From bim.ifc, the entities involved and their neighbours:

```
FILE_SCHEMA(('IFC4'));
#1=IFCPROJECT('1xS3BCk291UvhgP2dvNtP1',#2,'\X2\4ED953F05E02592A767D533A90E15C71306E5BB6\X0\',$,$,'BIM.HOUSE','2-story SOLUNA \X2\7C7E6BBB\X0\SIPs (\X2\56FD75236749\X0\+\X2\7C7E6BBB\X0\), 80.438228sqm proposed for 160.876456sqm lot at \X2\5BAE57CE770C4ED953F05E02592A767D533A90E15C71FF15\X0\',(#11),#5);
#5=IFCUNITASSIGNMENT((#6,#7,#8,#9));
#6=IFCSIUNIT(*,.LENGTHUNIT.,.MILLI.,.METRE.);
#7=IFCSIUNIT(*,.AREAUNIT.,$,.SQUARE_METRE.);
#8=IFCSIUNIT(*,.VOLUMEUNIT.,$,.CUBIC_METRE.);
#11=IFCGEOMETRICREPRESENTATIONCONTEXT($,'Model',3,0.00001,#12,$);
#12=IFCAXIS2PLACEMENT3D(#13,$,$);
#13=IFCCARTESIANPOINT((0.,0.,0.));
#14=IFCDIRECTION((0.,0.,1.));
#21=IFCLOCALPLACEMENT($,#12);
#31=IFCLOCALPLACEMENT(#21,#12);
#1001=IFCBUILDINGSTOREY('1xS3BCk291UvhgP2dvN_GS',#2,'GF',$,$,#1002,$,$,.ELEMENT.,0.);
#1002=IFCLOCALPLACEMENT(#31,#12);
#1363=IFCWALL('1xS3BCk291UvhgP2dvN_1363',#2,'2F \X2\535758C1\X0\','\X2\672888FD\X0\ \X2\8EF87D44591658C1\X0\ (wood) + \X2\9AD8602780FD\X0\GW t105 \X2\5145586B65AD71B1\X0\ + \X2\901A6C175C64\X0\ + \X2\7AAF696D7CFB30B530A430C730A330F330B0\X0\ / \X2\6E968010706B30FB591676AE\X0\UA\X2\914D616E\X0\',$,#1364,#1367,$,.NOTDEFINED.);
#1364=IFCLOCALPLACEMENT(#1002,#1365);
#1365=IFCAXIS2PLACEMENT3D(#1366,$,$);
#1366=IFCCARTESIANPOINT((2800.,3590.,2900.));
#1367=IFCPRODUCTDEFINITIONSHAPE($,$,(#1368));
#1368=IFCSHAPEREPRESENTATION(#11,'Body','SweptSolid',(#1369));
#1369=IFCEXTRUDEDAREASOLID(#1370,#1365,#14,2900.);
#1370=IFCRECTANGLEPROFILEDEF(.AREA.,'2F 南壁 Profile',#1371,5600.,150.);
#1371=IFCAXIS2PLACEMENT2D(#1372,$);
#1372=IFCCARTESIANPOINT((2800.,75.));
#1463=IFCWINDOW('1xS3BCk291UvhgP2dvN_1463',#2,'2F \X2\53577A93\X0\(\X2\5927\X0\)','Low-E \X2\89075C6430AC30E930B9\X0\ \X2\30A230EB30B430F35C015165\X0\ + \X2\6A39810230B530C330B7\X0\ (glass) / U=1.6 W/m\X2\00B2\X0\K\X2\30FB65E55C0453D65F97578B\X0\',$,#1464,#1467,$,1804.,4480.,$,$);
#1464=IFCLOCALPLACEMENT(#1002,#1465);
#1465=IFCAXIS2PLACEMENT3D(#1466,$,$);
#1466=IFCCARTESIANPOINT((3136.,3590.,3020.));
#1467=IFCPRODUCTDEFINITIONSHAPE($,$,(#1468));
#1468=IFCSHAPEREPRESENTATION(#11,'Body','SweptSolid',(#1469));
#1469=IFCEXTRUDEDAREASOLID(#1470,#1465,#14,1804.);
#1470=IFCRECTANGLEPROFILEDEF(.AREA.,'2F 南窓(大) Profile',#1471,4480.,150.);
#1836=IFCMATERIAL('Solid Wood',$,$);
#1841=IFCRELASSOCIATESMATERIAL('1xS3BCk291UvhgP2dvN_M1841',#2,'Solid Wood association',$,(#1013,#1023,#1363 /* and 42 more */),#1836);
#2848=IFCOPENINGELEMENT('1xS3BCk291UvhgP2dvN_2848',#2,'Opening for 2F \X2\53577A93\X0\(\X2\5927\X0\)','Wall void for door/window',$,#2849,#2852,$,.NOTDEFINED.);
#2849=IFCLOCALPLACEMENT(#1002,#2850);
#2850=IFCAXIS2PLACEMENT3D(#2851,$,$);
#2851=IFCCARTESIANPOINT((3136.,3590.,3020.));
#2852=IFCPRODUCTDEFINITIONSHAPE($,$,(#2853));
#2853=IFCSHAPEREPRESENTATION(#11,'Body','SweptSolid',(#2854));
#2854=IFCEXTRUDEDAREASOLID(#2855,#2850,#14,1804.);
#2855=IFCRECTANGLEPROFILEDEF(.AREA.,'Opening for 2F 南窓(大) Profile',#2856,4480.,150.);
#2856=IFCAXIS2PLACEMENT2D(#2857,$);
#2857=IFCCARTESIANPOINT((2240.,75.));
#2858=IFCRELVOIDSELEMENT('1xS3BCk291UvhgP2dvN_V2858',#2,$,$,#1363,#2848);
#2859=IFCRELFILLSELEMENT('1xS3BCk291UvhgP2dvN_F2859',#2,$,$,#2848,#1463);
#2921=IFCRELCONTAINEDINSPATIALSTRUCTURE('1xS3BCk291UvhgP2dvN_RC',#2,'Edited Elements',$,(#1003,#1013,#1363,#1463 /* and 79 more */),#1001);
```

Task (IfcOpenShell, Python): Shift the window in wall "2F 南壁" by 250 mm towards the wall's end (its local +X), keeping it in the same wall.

```python
import ifcopenshell
import ifcopenshell.api.geometry
import ifcopenshell.util.placement
import ifcopenshell.util.unit

model = ifcopenshell.open("bim.ifc")
unit_scale = ifcopenshell.util.unit.calculate_unit_scale(model)

window = model.by_guid("1xS3BCk291UvhgP2dvN_1463")
opening = window.FillsVoids[0].RelatingOpeningElement
wall = opening.VoidsElements[0].RelatingBuildingElement

wall_matrix = ifcopenshell.util.placement.get_local_placement(wall.ObjectPlacement)
shift = wall_matrix[:3, 0] * 0.25 / unit_scale
before = ifcopenshell.util.placement.get_local_placement(window.ObjectPlacement)[:3, 3].copy()

# The window is not placed relative to its opening, so move both.
for product in (opening, window):
    matrix = ifcopenshell.util.placement.get_local_placement(product.ObjectPlacement)
    matrix[:3, 3] += shift
    ifcopenshell.api.geometry.edit_object_placement(model, product=product, matrix=matrix, is_si=False)

after = ifcopenshell.util.placement.get_local_placement(window.ObjectPlacement)[:3, 3]
print("window moved by", (after - before).round(3) + 0.0)

model.write("bim_rev.ifc")
```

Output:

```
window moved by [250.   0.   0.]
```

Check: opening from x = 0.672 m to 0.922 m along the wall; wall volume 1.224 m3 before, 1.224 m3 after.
